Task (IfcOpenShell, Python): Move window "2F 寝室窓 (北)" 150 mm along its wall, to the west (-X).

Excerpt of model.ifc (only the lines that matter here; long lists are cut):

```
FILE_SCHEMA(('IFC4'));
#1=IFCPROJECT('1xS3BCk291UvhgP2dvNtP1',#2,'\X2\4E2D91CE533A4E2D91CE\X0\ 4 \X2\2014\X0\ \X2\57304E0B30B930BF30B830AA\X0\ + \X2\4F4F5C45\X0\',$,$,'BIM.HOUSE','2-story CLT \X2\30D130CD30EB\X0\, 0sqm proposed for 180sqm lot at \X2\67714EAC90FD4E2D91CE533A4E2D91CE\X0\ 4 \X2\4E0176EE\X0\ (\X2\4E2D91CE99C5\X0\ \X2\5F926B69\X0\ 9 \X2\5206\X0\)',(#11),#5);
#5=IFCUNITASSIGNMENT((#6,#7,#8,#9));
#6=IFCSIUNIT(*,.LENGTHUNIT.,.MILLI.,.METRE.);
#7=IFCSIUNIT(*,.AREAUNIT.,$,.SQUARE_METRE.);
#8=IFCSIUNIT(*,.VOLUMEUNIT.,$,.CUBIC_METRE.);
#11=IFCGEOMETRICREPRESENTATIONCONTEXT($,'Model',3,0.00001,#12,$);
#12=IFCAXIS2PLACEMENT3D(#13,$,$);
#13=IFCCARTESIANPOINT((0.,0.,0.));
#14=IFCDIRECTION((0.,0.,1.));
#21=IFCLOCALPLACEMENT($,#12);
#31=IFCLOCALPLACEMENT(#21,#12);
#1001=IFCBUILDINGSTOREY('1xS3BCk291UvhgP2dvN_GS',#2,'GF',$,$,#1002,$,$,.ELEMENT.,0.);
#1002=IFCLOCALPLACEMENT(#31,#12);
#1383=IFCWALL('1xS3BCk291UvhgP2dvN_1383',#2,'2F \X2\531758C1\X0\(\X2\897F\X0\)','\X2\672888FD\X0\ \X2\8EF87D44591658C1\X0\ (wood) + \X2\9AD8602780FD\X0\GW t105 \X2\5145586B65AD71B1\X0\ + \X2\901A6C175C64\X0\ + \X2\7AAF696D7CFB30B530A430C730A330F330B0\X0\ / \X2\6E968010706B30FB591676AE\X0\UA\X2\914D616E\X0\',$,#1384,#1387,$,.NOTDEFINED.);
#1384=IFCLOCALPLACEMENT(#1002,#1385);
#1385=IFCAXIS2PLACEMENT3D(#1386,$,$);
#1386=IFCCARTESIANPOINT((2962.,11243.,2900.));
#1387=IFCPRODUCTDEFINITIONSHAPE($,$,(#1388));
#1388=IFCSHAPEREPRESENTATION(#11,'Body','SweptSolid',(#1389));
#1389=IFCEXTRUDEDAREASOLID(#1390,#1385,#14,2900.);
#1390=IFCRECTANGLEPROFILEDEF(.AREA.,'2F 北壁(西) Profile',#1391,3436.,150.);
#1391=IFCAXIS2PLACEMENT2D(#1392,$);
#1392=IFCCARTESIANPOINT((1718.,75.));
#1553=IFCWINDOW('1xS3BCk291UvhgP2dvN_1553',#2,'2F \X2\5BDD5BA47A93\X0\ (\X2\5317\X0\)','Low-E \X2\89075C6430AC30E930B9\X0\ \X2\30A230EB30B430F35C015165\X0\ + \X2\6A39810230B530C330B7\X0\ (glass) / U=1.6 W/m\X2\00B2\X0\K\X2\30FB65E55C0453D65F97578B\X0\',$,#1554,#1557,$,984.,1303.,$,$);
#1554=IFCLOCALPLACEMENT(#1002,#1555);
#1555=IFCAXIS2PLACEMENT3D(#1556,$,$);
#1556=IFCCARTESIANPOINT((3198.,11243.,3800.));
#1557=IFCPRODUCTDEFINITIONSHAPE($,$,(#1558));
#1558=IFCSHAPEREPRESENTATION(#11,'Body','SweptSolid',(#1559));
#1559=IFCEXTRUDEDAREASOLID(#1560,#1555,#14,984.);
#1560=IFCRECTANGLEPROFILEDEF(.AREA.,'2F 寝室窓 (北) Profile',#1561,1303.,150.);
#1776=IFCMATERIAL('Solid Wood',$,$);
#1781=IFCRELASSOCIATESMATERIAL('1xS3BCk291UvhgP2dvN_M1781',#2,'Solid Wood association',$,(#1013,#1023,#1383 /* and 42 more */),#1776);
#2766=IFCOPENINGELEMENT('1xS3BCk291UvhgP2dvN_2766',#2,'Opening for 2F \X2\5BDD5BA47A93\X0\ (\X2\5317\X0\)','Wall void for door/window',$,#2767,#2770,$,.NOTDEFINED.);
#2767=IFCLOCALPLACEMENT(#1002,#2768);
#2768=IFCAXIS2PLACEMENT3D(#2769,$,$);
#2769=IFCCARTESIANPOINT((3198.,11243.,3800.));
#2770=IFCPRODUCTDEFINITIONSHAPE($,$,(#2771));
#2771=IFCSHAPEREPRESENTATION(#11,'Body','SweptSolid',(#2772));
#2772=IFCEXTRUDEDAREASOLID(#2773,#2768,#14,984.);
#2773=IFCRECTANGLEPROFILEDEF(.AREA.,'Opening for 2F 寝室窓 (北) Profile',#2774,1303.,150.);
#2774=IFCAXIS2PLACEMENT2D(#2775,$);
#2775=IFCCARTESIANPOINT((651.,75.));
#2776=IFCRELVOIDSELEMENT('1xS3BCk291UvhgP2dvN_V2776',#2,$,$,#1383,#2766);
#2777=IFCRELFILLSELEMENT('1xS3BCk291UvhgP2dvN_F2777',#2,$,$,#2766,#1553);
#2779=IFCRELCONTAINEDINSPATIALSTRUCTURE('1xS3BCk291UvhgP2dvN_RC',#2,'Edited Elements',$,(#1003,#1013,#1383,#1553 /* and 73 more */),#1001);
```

```python
import ifcopenshell
import ifcopenshell.api.geometry
import ifcopenshell.util.placement
import ifcopenshell.util.unit

model = ifcopenshell.open("model.ifc")
unit_scale = ifcopenshell.util.unit.calculate_unit_scale(model)

window = model.by_id(1553)
opening = window.FillsVoids[0].RelatingOpeningElement
wall = opening.VoidsElements[0].RelatingBuildingElement

wall_matrix = ifcopenshell.util.placement.get_local_placement(wall.ObjectPlacement)
shift = wall_matrix[:3, 0] * -0.15 / unit_scale
before = ifcopenshell.util.placement.get_local_placement(window.ObjectPlacement)[:3, 3].copy()

# The window is not placed relative to its opening, so move both.
for product in (opening, window):
    matrix = ifcopenshell.util.placement.get_local_placement(product.ObjectPlacement)
    matrix[:3, 3] += shift
    ifcopenshell.api.geometry.edit_object_placement(model, product=product, matrix=matrix, is_si=False)

after = ifcopenshell.util.placement.get_local_placement(window.ObjectPlacement)[:3, 3]
print("window moved by", (after - before).round(3) + 0.0)

model.write("model_v2.ifc")
```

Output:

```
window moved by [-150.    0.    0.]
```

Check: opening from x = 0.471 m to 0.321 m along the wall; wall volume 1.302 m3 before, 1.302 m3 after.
